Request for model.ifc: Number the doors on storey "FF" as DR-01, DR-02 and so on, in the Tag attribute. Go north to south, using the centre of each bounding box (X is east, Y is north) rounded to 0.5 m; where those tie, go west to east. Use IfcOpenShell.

First a look at what the model holds.

```python
import ifcopenshell
import ifcopenshell.util.element
import ifcopenshell.util.placement

model = ifcopenshell.open("model.ifc")
print(model.schema)
storey = next(s for s in model.by_type("IfcBuildingStorey") if s.Name == "FF")
doors = [e for e in ifcopenshell.util.element.get_decomposition(storey) if e.is_a("IfcDoor")]
for e in sorted(doors, key=lambda e: e.id()):
    origin = ifcopenshell.util.placement.get_local_placement(e.ObjectPlacement)[:3, 3]
    print(e.id(), e.Tag, e.Name, origin.round(2) + 0.0, sep=" | ")
```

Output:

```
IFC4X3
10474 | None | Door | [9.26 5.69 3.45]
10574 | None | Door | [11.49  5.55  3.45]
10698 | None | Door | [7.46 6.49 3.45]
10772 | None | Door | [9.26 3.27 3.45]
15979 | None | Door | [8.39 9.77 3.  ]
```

```python
import ifcopenshell
import ifcopenshell.geom
import ifcopenshell.util.element
import ifcopenshell.util.shape

model = ifcopenshell.open("model.ifc")
settings = ifcopenshell.geom.settings()
settings.set("use-world-coords", True)


def centre(element):
    shape = ifcopenshell.geom.create_shape(settings, element)
    return ifcopenshell.util.shape.get_bbox_centroid(shape.geometry)


storey = next(s for s in model.by_type("IfcBuildingStorey") if s.Name == "FF")
doors = [e for e in ifcopenshell.util.element.get_decomposition(storey) if e.is_a("IfcDoor")]

# Insertion points can sit at a corner or the storey origin, so sort by the geometry (in metres).
centres = {e: centre(e) for e in doors}
doors.sort(key=lambda e: (-round(centres[e][1] / 0.5), centres[e][0]))

for i, e in enumerate(doors, start=1):
    number = f"DR-{i:02d}"
    e.Tag = number
    print(e.id(), number)

model.write("model_rev.ifc")
```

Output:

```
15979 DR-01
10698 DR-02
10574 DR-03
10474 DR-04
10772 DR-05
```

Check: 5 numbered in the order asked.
